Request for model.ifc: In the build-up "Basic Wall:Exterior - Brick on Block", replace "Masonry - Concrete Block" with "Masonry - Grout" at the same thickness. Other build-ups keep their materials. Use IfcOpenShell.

First a look at what the model holds.

```python
import ifcopenshell
import ifcopenshell.util.element

model = ifcopenshell.open("model.ifc")
print(model.schema)
for layer_set in model.by_type("IfcMaterialLayerSet"):
    if layer_set.LayerSetName == "Basic Wall:Exterior - Brick on Block":
        for layer in layer_set.MaterialLayers:
            print(layer.id(), layer.Material and layer.Material.Name, layer.LayerThickness, sep=" | ")
        print(len(ifcopenshell.util.element.get_elements_by_material(model, layer_set)), "elements and types use it")
print(sorted(m.Name for m in model.by_type("IfcMaterial") if m.Name)[:60])
```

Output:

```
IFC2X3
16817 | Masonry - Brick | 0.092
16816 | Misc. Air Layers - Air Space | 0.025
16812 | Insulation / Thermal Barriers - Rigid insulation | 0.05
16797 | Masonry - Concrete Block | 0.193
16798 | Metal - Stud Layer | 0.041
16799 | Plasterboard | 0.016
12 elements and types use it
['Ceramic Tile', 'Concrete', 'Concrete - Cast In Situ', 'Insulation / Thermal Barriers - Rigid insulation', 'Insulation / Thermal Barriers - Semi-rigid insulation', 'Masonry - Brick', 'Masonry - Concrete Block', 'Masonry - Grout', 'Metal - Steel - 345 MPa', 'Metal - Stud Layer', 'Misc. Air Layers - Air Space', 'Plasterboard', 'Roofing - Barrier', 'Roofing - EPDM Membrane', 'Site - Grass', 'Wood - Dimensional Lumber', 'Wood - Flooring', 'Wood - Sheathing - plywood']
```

```python
import ifcopenshell
import ifcopenshell.api.material

model = ifcopenshell.open("model.ifc")

layer_set = next(s for s in model.by_type("IfcMaterialLayerSet") if s.LayerSetName == "Basic Wall:Exterior - Brick on Block")
layer = next(l for l in layer_set.MaterialLayers if l.Material and l.Material.Name == "Masonry - Concrete Block")
material = next(m for m in model.by_type("IfcMaterial") if m.Name == "Masonry - Grout")

# Point this one layer at the other material; renaming the old one would change it everywhere.
ifcopenshell.api.material.edit_layer(model, layer=layer, attributes={}, material=material)

print([l.Material.Name if l.Material else None for l in layer_set.MaterialLayers])

model.write("model-out.ifc")
```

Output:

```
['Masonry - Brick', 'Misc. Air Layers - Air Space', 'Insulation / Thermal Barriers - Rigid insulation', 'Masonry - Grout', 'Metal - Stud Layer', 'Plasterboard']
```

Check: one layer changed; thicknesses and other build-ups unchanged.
